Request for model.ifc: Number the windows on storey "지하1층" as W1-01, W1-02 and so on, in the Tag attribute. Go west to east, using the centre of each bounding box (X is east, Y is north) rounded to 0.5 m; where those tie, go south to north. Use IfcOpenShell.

First a look at what the model holds.

```python
import ifcopenshell
import ifcopenshell.util.element
import ifcopenshell.util.placement

model = ifcopenshell.open("model.ifc")
print(model.schema)
storey = next(s for s in model.by_type("IfcBuildingStorey") if s.Name == "지하1층")
windows = [e for e in ifcopenshell.util.element.get_decomposition(storey) if e.is_a("IfcWindow")]
for e in sorted(windows, key=lambda e: e.id()):
    origin = ifcopenshell.util.placement.get_local_placement(e.ObjectPlacement)[:3, 3]
    print(e.id(), e.Tag, e.Name, origin.round(2) + 0.0, sep=" | ")
```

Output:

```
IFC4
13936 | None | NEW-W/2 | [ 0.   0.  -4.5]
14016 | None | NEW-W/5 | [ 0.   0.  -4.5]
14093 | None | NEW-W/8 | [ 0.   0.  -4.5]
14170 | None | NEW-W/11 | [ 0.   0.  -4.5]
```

```python
import ifcopenshell
import ifcopenshell.geom
import ifcopenshell.util.element
import ifcopenshell.util.shape

model = ifcopenshell.open("model.ifc")
settings = ifcopenshell.geom.settings()
settings.set("use-world-coords", True)


def centre(element):
    shape = ifcopenshell.geom.create_shape(settings, element)
    return ifcopenshell.util.shape.get_bbox_centroid(shape.geometry)


storey = next(s for s in model.by_type("IfcBuildingStorey") if s.Name == "지하1층")
windows = [e for e in ifcopenshell.util.element.get_decomposition(storey) if e.is_a("IfcWindow")]

# Insertion points can sit at a corner or the storey origin, so sort by the geometry (in metres).
centres = {e: centre(e) for e in windows}
windows.sort(key=lambda e: (round(centres[e][0] / 0.5), centres[e][1]))

for i, e in enumerate(windows, start=1):
    number = f"W1-{i:02d}"
    e.Tag = number
    print(e.id(), number)

model.write("model_updated.ifc")
```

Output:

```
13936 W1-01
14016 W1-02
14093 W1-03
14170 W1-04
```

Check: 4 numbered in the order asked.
